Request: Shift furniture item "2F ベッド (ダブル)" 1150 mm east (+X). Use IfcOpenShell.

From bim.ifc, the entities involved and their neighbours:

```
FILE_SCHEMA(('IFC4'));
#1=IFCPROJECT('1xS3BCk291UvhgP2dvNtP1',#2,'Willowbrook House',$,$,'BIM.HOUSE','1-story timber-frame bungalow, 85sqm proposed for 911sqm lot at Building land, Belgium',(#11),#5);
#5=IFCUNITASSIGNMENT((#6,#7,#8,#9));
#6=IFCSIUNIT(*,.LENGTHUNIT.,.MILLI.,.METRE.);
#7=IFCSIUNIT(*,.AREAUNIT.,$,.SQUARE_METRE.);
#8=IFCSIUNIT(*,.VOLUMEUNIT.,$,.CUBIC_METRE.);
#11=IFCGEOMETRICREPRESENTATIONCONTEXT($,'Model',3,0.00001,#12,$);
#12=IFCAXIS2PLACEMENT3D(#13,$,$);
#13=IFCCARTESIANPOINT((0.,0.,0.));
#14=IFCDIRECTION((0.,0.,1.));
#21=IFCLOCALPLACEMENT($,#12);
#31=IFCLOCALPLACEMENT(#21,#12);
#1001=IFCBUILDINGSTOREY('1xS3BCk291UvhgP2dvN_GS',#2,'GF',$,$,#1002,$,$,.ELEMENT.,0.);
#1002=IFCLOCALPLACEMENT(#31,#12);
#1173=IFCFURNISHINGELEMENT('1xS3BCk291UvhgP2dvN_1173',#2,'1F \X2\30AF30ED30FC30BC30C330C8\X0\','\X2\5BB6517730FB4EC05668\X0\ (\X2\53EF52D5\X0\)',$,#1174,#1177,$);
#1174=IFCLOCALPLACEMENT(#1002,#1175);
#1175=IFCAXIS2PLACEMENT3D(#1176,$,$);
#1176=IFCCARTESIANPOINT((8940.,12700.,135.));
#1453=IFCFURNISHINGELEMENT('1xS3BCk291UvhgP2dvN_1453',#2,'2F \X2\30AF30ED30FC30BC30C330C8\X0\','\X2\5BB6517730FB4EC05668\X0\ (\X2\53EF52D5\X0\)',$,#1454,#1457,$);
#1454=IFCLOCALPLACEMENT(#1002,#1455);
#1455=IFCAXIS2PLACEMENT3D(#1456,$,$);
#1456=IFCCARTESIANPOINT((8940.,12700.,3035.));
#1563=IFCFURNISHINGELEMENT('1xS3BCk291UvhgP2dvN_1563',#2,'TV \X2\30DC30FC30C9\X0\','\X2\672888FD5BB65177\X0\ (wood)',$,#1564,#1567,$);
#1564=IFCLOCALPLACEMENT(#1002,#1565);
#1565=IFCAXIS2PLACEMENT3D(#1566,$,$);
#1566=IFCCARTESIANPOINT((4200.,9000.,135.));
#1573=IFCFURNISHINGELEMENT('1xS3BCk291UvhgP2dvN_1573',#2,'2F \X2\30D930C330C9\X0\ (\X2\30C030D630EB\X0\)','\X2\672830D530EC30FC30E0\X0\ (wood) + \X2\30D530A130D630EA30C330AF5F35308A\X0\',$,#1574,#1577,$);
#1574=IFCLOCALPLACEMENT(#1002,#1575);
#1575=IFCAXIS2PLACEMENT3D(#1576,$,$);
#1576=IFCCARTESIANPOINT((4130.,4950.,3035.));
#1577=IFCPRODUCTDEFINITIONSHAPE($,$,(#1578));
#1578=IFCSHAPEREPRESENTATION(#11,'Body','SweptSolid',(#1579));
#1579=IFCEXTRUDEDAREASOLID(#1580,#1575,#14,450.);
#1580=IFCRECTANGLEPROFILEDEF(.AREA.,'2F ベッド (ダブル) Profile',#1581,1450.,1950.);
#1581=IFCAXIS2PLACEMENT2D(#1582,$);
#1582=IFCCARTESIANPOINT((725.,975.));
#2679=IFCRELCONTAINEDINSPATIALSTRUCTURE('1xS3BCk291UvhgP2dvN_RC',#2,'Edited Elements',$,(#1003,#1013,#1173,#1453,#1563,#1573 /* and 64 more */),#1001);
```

```python
import ifcopenshell
import ifcopenshell.api.geometry
import ifcopenshell.util.placement
import ifcopenshell.util.unit

model = ifcopenshell.open("bim.ifc")
unit_scale = ifcopenshell.util.unit.calculate_unit_scale(model)

item = model.by_guid("1xS3BCk291UvhgP2dvN_1573")
matrix = ifcopenshell.util.placement.get_local_placement(item.ObjectPlacement)
matrix[0, 3] += 1.15 / unit_scale
ifcopenshell.api.geometry.edit_object_placement(model, product=item, matrix=matrix, is_si=False)

print(ifcopenshell.util.placement.get_local_placement(item.ObjectPlacement).round(3) + 0.0)

model.write("bim_edited.ifc")
```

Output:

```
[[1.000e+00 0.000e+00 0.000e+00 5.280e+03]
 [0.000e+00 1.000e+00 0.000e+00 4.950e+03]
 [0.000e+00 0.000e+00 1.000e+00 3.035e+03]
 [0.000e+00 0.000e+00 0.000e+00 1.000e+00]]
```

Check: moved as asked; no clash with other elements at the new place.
